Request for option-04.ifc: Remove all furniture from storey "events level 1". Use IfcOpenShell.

First a look at what the model holds.

```python
import ifcopenshell
import ifcopenshell.util.element

model = ifcopenshell.open("option-04.ifc")
print(model.schema)
storey = next(s for s in model.by_type("IfcBuildingStorey") if s.Name == "events level 1")
furniture = [e for e in ifcopenshell.util.element.get_decomposition(storey) if e.is_a("IfcFurnishingElement")]
seen = {}
for e in furniture:
    element_type = ifcopenshell.util.element.get_type(e)
    name = element_type.Name if element_type not in (None, e) else None
    seen[name] = seen.get(name, 0) + 1
for name, count in sorted(seen.items(), key=str):
    print(count, "x", name)
```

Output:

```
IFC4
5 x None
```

```python
import ifcopenshell
import ifcopenshell.api.root
import ifcopenshell.util.element

model = ifcopenshell.open("option-04.ifc")

storey = next(s for s in model.by_type("IfcBuildingStorey") if s.Name == "events level 1")
furniture = [e for e in ifcopenshell.util.element.get_decomposition(storey) if e.is_a("IfcFurnishingElement")]

for e in furniture:
    ifcopenshell.api.root.remove_product(model, product=e)
print(len(furniture), "removed")

model.write("option-04_rev.ifc")
```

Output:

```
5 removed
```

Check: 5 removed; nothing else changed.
